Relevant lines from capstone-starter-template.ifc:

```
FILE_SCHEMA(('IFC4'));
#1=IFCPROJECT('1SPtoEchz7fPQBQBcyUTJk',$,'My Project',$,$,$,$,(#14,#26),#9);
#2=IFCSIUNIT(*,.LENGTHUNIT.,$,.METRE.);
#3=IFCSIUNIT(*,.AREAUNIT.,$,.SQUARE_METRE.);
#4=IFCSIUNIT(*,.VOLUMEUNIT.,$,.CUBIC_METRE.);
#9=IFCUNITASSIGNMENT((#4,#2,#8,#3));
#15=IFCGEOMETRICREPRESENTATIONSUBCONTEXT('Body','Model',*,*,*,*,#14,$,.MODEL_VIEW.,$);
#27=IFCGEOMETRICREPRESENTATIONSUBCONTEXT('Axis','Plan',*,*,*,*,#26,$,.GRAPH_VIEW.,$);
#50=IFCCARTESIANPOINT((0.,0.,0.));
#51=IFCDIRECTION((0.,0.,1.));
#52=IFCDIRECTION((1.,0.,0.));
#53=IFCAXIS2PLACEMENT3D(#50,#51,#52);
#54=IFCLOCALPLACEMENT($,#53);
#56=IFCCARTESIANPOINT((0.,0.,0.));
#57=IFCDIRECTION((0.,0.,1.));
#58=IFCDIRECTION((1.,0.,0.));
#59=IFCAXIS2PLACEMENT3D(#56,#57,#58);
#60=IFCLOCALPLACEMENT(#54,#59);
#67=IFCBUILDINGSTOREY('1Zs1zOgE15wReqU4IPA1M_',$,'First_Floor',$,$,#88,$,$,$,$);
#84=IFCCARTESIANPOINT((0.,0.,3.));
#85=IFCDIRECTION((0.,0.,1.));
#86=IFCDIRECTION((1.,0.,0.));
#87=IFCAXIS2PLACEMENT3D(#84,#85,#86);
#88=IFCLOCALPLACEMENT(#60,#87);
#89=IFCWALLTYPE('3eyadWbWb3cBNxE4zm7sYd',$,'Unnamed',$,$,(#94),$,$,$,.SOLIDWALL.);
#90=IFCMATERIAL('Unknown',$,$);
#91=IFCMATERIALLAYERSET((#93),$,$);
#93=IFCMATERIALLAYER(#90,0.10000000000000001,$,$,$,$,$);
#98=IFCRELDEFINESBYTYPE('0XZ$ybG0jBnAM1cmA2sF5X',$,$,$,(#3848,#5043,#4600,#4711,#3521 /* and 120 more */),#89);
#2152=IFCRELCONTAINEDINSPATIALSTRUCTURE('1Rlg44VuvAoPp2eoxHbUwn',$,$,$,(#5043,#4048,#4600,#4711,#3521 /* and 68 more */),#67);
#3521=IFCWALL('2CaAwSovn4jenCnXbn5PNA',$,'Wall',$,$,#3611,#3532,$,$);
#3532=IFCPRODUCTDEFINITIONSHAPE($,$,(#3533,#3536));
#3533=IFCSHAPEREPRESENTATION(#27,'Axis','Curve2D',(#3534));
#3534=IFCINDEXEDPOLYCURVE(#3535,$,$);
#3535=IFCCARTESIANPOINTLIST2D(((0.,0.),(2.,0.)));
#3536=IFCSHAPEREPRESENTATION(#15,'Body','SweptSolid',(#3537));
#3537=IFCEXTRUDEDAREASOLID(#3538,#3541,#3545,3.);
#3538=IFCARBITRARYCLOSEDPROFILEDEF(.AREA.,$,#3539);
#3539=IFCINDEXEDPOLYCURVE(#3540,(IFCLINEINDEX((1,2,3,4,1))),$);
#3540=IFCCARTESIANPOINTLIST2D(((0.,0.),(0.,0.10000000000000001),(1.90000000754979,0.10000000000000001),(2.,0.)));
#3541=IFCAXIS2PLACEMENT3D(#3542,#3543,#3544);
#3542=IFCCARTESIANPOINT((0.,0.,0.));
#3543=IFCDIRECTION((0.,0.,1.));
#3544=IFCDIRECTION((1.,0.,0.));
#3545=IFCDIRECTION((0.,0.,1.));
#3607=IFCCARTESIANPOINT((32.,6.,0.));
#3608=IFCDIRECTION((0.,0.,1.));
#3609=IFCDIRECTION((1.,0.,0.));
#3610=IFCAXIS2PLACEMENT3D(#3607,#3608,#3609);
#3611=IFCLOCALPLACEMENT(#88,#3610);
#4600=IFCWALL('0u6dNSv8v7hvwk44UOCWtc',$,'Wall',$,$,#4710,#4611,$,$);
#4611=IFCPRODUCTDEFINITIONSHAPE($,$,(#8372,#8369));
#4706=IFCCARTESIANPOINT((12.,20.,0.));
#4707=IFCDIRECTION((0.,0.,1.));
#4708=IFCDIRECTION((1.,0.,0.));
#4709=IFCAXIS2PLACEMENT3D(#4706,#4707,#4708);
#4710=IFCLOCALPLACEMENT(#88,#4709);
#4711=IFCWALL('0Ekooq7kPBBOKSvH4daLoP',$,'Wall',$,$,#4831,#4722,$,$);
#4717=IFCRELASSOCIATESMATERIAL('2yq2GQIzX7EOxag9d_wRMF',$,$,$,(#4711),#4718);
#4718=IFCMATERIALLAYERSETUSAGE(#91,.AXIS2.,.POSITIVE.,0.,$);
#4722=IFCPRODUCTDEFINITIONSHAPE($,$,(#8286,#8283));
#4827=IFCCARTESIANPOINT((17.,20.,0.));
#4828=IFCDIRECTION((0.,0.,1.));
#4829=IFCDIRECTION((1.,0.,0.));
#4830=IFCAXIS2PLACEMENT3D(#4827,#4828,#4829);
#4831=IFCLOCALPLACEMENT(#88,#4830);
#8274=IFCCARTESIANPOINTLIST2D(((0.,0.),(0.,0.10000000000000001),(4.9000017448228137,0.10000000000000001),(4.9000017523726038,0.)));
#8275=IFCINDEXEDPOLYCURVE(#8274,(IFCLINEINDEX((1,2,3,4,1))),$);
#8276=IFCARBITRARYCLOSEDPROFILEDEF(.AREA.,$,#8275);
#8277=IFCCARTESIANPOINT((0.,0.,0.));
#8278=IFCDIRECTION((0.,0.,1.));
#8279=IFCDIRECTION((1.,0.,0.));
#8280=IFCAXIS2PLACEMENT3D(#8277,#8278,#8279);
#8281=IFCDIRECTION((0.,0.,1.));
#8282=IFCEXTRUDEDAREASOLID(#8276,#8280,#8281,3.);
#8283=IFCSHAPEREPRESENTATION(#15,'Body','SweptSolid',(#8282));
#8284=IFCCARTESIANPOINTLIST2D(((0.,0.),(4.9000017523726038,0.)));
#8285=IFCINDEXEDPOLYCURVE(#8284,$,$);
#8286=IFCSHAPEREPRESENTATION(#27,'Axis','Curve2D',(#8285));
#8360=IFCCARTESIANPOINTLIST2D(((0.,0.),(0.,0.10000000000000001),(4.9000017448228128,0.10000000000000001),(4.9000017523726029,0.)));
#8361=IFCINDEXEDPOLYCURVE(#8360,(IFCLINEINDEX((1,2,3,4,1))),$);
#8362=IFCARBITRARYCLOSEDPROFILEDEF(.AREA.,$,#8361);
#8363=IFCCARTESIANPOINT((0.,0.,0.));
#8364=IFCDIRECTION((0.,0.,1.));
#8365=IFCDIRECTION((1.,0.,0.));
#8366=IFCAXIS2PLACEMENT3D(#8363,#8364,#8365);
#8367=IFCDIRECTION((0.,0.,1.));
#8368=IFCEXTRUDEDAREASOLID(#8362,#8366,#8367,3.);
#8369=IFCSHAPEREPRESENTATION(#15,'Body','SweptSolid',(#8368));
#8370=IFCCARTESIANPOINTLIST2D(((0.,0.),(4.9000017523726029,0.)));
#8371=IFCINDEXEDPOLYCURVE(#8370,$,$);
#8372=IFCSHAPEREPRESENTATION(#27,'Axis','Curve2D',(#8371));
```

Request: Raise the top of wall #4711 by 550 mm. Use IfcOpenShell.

```python
import ifcopenshell
import ifcopenshell.geom
import ifcopenshell.util.representation
import ifcopenshell.util.shape
import ifcopenshell.util.unit

model = ifcopenshell.open("capstone-starter-template.ifc")
unit_scale = ifcopenshell.util.unit.calculate_unit_scale(model)
settings = ifcopenshell.geom.settings()


def volume(element):
    """Net volume in cubic metres, openings subtracted."""
    shape = ifcopenshell.geom.create_shape(settings, element)
    return ifcopenshell.util.shape.get_volume(shape.geometry)


wall = model.by_guid("0Ekooq7kPBBOKSvH4daLoP")
before = volume(wall)

body = ifcopenshell.util.representation.get_representation(wall, "Model", "Body")
solid = body.Items[0]
old_height = solid.Depth
solid.Depth += 0.55 / unit_scale
after = volume(wall)

print(f"height {old_height:g} -> {solid.Depth:g}, volume {before:.3f} -> {after:.3f} m3")

model.write("capstone-starter-template_rev.ifc")
```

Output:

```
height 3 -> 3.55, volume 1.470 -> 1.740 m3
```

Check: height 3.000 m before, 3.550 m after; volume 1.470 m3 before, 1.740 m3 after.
